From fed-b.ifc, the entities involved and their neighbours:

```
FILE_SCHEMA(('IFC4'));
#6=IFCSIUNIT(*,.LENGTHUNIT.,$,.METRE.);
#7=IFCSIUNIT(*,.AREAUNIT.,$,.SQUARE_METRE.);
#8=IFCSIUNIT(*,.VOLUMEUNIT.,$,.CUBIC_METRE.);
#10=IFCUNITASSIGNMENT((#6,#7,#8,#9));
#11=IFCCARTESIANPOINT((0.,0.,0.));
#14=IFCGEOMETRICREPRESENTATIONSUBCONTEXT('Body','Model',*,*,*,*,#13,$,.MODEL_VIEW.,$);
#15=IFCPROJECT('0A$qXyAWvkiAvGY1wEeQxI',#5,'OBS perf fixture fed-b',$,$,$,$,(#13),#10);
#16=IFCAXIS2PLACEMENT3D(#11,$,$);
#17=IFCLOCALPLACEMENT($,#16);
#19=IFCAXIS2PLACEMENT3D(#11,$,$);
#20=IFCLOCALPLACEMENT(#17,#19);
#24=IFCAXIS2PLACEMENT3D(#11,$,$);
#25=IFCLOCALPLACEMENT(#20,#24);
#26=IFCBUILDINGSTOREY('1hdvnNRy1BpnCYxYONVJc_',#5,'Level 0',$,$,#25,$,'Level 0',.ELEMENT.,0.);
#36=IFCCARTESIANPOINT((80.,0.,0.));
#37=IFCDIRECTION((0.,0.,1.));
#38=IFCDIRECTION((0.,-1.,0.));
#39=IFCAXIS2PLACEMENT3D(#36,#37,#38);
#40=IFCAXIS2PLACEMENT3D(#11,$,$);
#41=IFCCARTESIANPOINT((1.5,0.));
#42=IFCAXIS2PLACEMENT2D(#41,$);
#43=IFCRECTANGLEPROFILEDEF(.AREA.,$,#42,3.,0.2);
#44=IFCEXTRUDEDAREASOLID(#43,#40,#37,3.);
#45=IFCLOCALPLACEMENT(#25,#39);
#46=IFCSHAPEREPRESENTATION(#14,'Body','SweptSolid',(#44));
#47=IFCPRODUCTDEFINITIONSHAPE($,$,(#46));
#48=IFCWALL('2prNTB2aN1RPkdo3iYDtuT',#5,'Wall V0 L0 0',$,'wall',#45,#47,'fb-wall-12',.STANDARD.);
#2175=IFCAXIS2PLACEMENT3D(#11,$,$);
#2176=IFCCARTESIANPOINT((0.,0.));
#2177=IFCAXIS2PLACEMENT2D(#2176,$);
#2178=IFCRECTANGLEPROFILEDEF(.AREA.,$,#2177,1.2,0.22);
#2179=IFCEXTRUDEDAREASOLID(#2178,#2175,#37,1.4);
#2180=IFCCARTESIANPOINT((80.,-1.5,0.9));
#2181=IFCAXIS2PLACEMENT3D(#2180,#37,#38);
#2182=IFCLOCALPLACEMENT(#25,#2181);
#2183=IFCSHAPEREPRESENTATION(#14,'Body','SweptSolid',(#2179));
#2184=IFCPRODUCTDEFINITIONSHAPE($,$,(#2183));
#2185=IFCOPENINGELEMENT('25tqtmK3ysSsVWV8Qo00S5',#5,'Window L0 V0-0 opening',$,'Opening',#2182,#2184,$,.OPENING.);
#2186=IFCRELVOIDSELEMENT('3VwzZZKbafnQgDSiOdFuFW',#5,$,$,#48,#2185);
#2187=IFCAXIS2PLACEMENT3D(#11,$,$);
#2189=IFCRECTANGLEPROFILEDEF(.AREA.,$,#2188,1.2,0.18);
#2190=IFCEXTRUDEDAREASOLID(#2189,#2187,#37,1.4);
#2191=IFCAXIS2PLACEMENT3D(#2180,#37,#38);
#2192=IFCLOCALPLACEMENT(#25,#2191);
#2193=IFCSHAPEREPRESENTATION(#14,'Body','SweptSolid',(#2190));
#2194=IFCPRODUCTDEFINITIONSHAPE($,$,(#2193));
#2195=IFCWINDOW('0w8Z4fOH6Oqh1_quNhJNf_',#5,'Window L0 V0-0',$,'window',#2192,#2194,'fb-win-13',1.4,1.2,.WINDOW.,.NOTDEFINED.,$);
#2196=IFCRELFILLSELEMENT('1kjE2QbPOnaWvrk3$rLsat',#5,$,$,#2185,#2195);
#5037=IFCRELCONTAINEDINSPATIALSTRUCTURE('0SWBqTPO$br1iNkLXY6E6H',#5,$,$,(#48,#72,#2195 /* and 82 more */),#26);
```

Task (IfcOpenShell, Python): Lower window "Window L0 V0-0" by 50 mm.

```python
import numpy as np
import ifcopenshell
import ifcopenshell.api.geometry
import ifcopenshell.util.placement
import ifcopenshell.util.unit

model = ifcopenshell.open("fed-b.ifc")
unit_scale = ifcopenshell.util.unit.calculate_unit_scale(model)

window = model.by_guid("0w8Z4fOH6Oqh1_quNhJNf_")
opening = window.FillsVoids[0].RelatingOpeningElement
dz = -0.05 / unit_scale

shift = np.array([0.0, 0.0, dz])
# The window is not placed relative to its opening, so move both.
for product in (opening, window):
    matrix = ifcopenshell.util.placement.get_local_placement(product.ObjectPlacement)
    matrix[:3, 3] += shift
    ifcopenshell.api.geometry.edit_object_placement(model, product=product, matrix=matrix, is_si=False)

print(f"moved by {dz * unit_scale:+.3f} m")

model.write("fed-b_rev.ifc")
```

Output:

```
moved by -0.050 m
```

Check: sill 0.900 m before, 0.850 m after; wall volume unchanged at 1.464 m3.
